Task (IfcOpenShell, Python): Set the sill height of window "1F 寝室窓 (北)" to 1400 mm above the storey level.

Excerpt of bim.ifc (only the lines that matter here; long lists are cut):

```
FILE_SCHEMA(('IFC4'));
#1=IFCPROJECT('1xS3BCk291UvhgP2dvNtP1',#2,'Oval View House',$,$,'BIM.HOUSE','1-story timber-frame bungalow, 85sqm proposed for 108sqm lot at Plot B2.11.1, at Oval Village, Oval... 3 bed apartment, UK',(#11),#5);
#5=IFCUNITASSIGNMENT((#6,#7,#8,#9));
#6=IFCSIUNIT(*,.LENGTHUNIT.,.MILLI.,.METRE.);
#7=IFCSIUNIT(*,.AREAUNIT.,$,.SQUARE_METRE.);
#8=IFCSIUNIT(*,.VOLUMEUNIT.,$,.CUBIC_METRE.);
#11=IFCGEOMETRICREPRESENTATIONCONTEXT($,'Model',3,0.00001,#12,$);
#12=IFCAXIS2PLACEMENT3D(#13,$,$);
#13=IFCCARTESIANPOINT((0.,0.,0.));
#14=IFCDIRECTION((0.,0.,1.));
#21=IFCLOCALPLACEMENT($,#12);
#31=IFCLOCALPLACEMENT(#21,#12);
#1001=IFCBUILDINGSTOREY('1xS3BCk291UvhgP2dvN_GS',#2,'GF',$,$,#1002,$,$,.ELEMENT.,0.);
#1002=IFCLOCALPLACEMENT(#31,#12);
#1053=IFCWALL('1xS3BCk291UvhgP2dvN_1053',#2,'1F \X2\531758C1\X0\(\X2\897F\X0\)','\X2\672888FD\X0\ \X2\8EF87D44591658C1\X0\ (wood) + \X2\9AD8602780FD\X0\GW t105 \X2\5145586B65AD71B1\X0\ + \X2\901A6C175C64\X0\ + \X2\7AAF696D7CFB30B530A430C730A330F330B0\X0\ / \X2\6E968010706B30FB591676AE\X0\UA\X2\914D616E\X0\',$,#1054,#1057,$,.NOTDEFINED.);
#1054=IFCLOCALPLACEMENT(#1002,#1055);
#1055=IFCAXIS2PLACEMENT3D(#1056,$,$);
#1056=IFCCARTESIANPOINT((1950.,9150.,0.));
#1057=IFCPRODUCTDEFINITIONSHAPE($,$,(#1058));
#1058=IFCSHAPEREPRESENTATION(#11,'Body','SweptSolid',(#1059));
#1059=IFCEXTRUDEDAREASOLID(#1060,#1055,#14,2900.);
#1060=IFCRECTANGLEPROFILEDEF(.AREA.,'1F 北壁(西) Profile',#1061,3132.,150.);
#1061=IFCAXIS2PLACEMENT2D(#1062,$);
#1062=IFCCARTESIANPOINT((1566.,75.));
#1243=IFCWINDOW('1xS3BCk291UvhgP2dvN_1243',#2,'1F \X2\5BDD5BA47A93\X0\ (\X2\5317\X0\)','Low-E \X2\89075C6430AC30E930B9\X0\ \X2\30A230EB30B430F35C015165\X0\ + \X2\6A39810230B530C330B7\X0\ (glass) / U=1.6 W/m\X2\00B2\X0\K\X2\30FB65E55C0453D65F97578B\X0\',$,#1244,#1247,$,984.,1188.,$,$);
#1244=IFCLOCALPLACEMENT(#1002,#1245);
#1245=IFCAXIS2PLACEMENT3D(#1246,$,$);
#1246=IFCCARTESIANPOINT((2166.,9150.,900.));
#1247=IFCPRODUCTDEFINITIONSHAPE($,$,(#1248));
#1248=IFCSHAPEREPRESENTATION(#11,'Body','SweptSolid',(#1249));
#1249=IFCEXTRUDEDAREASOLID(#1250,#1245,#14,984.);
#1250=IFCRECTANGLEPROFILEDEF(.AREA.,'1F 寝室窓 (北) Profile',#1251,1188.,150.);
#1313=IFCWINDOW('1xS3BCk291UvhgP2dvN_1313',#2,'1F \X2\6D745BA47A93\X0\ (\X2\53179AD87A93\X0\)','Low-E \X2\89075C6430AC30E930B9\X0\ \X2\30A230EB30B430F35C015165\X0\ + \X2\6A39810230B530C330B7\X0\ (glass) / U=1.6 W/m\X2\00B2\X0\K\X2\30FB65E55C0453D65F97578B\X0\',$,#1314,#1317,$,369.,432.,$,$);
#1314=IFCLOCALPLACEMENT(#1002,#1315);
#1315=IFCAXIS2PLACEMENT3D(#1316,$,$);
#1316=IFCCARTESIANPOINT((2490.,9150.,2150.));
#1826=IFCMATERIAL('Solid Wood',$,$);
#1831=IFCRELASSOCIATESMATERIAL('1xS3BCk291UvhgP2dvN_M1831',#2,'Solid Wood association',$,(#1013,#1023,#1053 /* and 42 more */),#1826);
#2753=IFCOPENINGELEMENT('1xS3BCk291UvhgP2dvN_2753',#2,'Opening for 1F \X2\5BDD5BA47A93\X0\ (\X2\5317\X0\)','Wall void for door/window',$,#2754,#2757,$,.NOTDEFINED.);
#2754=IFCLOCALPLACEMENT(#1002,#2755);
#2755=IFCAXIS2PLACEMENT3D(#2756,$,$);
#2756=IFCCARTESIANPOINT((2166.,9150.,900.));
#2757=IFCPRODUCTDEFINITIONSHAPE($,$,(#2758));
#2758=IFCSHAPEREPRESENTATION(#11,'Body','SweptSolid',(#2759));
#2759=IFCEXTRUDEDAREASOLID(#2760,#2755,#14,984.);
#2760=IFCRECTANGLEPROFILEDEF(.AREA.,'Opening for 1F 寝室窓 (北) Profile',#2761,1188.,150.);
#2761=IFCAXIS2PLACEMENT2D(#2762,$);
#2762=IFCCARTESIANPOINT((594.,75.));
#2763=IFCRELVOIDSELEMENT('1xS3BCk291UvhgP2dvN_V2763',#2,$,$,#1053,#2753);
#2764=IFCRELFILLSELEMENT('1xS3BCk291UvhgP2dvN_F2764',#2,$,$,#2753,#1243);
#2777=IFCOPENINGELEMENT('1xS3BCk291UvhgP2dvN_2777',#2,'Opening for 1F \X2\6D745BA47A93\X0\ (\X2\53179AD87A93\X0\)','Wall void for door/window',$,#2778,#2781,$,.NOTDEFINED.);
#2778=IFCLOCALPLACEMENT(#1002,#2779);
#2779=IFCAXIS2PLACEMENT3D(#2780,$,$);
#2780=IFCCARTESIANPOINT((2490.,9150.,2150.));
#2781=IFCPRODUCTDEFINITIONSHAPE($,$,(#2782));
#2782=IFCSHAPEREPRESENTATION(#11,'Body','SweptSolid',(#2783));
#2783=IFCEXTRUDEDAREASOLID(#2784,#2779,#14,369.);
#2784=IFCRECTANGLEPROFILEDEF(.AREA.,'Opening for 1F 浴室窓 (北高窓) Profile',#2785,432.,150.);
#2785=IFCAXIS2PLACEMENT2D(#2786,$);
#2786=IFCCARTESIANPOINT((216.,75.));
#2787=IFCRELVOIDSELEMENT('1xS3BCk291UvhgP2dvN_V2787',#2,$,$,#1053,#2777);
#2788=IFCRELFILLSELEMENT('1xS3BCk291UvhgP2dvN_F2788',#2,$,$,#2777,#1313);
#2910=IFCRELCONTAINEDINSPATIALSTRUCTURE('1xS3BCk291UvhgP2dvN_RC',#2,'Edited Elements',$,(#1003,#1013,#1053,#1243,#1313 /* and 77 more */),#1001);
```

```python
import numpy as np
import ifcopenshell
import ifcopenshell.api.geometry
import ifcopenshell.geom
import ifcopenshell.util.element
import ifcopenshell.util.placement
import ifcopenshell.util.shape
import ifcopenshell.util.unit

model = ifcopenshell.open("bim.ifc")
unit_scale = ifcopenshell.util.unit.calculate_unit_scale(model)

window = model.by_guid("1xS3BCk291UvhgP2dvN_1243")
opening = window.FillsVoids[0].RelatingOpeningElement
storey = ifcopenshell.util.element.get_container(window, ifc_class="IfcBuildingStorey")
level = ifcopenshell.util.placement.get_local_placement(storey.ObjectPlacement)[2, 3]

# The opening's origin need not be at the sill, so measure its lowest point.
shape = ifcopenshell.geom.create_shape(ifcopenshell.geom.settings(), opening)
bottom = ifcopenshell.util.shape.get_shape_bottom_elevation(shape, shape.geometry) / unit_scale
dz = level + 1.4 / unit_scale - bottom

shift = np.array([0.0, 0.0, dz])
# The window is not placed relative to its opening, so move both.
for product in (opening, window):
    matrix = ifcopenshell.util.placement.get_local_placement(product.ObjectPlacement)
    matrix[:3, 3] += shift
    ifcopenshell.api.geometry.edit_object_placement(model, product=product, matrix=matrix, is_si=False)

print(f"moved by {dz * unit_scale:+.3f} m")

model.write("bim_v2.ifc")
```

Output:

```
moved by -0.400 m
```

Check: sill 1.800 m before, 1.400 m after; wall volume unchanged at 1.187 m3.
